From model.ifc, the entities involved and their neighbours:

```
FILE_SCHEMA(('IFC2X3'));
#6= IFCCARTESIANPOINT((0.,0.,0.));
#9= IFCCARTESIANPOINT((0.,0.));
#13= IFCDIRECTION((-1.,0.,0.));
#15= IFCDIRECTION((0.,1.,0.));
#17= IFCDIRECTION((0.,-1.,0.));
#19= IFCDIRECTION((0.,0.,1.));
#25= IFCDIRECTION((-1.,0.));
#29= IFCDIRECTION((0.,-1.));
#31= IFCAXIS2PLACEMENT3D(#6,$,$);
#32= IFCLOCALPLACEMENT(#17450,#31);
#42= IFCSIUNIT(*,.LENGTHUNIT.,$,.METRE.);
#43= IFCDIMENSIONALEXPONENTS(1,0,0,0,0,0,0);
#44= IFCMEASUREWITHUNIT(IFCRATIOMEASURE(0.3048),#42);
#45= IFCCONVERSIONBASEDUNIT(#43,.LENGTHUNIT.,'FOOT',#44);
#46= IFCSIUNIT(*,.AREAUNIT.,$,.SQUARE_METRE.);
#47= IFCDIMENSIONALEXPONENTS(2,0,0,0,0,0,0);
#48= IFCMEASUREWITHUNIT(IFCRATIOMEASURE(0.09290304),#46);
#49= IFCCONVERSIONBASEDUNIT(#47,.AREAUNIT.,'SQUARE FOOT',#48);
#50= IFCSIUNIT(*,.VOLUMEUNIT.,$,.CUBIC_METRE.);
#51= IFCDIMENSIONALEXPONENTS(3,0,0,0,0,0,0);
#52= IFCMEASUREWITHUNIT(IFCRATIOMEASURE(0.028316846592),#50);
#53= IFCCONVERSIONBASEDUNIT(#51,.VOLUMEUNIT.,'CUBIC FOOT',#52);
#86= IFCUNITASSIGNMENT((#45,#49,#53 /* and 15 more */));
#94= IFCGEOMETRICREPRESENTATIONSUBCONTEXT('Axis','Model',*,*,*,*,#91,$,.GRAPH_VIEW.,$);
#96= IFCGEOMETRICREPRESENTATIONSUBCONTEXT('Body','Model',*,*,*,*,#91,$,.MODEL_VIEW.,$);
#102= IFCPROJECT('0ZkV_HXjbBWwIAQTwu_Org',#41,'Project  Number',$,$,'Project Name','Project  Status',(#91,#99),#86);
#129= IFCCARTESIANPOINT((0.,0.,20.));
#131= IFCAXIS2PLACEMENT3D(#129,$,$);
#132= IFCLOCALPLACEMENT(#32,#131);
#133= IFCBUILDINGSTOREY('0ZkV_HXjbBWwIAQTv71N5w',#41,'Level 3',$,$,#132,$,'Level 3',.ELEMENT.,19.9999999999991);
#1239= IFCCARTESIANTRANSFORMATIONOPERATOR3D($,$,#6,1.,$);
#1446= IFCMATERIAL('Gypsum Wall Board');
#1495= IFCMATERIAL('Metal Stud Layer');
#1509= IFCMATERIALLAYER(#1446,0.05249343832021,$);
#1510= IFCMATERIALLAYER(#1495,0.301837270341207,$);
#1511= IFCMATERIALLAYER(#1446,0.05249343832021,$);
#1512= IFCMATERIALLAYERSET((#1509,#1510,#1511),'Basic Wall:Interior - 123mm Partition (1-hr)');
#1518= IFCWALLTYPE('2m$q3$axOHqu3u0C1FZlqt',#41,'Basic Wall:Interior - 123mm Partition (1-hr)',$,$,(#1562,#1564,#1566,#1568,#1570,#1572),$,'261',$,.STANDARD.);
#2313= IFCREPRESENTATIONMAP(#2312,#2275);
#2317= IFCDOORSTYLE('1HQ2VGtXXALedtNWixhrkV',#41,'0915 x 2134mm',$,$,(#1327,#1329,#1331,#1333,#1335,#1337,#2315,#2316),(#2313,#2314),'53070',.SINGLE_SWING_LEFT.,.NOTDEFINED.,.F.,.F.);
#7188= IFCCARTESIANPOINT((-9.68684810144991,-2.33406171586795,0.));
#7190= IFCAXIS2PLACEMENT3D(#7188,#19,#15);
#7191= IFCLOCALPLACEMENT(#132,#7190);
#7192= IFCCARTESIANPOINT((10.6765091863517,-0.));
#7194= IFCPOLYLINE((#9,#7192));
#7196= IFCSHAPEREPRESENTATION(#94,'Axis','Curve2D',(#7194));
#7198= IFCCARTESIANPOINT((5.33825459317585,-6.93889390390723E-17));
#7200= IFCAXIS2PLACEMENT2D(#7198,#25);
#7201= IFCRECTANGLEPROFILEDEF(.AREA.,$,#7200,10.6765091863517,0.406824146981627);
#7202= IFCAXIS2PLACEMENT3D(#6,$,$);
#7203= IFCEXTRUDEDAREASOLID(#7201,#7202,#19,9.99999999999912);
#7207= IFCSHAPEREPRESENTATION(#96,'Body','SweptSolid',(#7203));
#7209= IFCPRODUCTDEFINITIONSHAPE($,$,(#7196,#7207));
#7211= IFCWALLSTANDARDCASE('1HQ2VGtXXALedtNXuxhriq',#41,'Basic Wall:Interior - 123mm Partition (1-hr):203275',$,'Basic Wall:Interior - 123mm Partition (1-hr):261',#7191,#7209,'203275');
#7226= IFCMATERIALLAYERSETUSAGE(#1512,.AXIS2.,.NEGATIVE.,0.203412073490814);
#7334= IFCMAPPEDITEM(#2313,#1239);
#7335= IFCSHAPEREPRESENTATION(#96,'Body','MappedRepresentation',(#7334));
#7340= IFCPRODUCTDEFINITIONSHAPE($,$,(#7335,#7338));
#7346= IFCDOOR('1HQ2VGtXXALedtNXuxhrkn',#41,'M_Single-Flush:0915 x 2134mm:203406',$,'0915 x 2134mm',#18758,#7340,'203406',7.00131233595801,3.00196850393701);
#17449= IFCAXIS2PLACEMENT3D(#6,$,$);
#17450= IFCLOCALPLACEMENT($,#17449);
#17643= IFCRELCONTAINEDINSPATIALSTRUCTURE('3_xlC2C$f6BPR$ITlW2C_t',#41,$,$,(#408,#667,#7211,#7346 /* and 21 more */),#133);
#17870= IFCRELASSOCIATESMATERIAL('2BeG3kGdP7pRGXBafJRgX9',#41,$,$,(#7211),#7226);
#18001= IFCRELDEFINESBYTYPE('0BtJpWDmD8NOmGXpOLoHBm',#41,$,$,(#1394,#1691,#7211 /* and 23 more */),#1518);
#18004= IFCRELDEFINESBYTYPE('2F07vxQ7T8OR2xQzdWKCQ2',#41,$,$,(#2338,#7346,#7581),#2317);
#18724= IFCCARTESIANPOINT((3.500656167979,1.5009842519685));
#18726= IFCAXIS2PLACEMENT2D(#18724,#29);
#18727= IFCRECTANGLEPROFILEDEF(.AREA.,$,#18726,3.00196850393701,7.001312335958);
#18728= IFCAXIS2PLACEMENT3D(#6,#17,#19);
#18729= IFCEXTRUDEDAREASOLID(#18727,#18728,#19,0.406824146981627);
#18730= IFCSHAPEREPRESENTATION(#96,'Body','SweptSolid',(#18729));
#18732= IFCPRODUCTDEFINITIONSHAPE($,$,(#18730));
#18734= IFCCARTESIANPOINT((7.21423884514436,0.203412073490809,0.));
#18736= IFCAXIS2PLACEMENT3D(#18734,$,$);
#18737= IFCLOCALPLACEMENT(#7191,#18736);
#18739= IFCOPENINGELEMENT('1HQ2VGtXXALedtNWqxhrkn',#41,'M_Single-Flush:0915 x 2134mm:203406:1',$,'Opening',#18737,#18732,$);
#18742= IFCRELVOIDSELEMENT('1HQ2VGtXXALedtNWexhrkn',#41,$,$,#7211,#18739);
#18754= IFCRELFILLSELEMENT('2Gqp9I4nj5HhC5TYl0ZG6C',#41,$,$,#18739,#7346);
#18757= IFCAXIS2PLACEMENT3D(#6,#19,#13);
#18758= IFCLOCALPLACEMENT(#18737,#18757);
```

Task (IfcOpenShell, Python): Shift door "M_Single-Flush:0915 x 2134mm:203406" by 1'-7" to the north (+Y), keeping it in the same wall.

```python
import ifcopenshell
import ifcopenshell.api.geometry
import ifcopenshell.util.placement
import ifcopenshell.util.unit

model = ifcopenshell.open("model.ifc")
unit_scale = ifcopenshell.util.unit.calculate_unit_scale(model)

door = model.by_guid("1HQ2VGtXXALedtNXuxhrkn")
opening = door.FillsVoids[0].RelatingOpeningElement
wall = opening.VoidsElements[0].RelatingBuildingElement

wall_matrix = ifcopenshell.util.placement.get_local_placement(wall.ObjectPlacement)
shift = wall_matrix[:3, 0] * 19 * 0.0254 / unit_scale
before = ifcopenshell.util.placement.get_local_placement(door.ObjectPlacement)[:3, 3].copy()

# The door is placed relative to its opening, so it follows when the opening moves.
matrix = ifcopenshell.util.placement.get_local_placement(opening.ObjectPlacement)
matrix[:3, 3] += shift
ifcopenshell.api.geometry.edit_object_placement(
    model, product=opening, matrix=matrix, is_si=False, should_transform_children=True
)

after = ifcopenshell.util.placement.get_local_placement(door.ObjectPlacement)[:3, 3]
print("door moved by", (after - before).round(3) + 0.0)

model.write("model_edited.ifc")
```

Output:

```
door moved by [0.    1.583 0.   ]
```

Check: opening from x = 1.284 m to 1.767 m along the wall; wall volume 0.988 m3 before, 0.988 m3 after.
